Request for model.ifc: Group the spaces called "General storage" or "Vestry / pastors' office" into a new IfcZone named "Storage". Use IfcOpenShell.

First a look at what the model holds.

```python
import ifcopenshell

model = ifcopenshell.open("model.ifc")
print(model.schema)
seen = {}
for space in model.by_type("IfcSpace"):
    seen[space.LongName] = seen.get(space.LongName, 0) + 1
for name, count in sorted(seen.items(), key=str):
    print(count, "x", name)
print("zones:", [z.Name for z in model.by_type("IfcZone")][:20])
```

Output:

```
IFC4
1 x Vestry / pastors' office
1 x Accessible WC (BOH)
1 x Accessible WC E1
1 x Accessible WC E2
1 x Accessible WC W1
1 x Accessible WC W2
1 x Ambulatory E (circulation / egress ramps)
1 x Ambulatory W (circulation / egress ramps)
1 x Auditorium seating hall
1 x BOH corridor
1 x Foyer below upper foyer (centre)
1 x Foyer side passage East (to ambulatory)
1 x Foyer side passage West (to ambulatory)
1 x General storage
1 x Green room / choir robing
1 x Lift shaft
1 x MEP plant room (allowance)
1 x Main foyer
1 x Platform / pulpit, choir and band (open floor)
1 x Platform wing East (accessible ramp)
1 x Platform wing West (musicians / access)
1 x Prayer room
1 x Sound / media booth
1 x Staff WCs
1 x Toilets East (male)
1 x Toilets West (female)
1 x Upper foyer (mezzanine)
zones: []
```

```python
import ifcopenshell
import ifcopenshell.api.group
import ifcopenshell.api.root

model = ifcopenshell.open("model.ifc")

names = {"General storage", "Vestry / pastors' office"}
spaces = [s for s in model.by_type("IfcSpace") if s.LongName in names]

zone = ifcopenshell.api.root.create_entity(model, ifc_class="IfcZone", name="Storage")
ifcopenshell.api.group.assign_group(model, products=spaces, group=zone)
print(len(spaces), "spaces in", zone.Name)

model.write("model_v2.ifc")
```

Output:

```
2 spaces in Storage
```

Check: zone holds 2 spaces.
